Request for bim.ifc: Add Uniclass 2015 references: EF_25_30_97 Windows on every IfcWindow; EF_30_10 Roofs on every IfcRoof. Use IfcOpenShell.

First a look at what the model holds.

```python
import ifcopenshell

model = ifcopenshell.open("bim.ifc")
print(model.schema)
print("classifications:", [c.Name for c in model.by_type("IfcClassification")])
for ifc_class in ("IfcDoor", "IfcRoof", "IfcStair", "IfcWall", "IfcWindow"):
    print(ifc_class, len(model.by_type(ifc_class)))
```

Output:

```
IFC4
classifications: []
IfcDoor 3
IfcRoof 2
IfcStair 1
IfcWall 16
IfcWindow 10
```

```python
import ifcopenshell
import ifcopenshell.api.classification

model = ifcopenshell.open("bim.ifc")

system = ifcopenshell.api.classification.add_classification(model, classification="Uniclass 2015")

codes = {
    "IfcWindow": ("EF_25_30_97", "Windows"),
    "IfcRoof": ("EF_30_10", "Roofs"),
}
for ifc_class, (code, name) in codes.items():
    products = model.by_type(ifc_class)
    ifcopenshell.api.classification.add_reference(
        model, products=products, classification=system, identification=code, name=name
    )
    print(code, len(products))

model.write("bim_rev.ifc")
```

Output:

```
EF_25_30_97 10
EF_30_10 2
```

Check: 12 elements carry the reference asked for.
